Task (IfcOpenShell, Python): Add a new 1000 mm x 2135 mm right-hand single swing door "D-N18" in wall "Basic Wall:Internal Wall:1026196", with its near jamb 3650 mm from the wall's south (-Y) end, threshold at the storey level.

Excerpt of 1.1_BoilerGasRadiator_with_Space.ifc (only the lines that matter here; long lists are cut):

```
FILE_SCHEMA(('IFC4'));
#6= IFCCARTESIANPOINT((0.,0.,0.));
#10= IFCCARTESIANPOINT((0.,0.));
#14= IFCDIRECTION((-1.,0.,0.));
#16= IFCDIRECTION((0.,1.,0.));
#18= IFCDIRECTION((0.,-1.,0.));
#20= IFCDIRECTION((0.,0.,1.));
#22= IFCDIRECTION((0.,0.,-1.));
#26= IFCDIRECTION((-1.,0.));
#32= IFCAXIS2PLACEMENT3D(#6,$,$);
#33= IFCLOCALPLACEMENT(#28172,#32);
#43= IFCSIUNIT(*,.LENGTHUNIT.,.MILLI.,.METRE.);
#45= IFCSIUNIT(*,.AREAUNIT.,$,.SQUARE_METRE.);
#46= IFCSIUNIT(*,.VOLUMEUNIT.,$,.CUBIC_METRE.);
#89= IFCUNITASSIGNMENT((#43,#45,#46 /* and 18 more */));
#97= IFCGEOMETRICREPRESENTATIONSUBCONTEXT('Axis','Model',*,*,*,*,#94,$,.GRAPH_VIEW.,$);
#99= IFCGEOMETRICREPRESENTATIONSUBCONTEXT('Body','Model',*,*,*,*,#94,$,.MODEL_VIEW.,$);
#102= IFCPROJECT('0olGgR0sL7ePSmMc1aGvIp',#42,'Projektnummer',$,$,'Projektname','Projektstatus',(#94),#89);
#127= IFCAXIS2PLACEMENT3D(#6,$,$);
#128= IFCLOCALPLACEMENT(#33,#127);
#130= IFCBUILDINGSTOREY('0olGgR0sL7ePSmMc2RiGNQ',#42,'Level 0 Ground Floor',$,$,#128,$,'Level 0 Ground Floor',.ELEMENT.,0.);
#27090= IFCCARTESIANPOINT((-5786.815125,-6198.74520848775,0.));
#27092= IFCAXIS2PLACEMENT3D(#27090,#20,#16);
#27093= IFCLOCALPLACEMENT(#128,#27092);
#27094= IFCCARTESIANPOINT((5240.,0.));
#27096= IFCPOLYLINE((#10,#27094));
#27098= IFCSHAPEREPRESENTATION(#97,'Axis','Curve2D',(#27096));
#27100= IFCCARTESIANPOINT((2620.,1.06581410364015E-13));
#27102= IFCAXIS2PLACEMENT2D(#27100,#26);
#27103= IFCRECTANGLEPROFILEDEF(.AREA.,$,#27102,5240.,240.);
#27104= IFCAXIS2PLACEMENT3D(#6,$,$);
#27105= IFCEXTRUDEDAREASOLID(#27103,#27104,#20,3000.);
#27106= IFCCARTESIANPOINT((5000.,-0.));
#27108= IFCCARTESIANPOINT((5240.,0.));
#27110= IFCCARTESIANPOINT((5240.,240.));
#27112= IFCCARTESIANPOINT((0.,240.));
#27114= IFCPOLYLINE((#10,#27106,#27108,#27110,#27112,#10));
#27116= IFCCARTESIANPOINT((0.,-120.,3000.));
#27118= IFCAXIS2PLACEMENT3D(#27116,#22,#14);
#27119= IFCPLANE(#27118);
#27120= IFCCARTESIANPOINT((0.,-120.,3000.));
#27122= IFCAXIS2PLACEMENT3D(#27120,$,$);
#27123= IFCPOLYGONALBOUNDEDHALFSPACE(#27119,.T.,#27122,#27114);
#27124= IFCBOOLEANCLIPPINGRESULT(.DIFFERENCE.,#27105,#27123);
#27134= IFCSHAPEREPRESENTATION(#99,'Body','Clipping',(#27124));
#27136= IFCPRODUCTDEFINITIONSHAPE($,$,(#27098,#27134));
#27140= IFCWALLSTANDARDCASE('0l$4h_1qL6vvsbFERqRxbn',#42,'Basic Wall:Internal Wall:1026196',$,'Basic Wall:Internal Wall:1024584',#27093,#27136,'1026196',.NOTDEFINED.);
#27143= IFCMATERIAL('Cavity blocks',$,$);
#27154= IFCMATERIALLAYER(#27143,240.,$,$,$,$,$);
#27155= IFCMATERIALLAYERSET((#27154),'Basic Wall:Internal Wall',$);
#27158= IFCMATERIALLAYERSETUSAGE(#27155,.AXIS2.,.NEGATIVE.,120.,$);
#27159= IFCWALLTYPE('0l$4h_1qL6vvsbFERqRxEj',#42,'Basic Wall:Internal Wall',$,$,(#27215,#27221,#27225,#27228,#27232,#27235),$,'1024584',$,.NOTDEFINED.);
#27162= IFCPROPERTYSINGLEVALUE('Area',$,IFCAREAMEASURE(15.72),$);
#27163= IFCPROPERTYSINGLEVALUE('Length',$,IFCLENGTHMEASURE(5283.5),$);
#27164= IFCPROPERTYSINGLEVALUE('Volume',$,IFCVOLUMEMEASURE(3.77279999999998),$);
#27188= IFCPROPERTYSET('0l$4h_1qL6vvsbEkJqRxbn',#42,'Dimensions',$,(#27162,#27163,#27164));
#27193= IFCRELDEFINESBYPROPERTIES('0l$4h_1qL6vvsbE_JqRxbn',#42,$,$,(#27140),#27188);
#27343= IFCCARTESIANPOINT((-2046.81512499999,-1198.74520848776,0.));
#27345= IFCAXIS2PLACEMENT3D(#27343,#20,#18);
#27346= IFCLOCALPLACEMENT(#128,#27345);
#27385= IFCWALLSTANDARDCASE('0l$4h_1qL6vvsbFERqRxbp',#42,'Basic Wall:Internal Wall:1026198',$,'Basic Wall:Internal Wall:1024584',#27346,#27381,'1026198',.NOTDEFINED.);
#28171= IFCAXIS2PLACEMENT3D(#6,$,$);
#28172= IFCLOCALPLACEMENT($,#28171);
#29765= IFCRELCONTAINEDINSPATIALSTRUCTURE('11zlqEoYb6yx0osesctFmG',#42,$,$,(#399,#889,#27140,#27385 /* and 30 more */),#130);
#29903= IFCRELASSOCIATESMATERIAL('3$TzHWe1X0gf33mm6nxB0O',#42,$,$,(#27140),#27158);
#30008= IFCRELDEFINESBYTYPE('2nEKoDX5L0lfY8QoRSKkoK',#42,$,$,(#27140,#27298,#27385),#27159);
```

```python
import numpy as np
import ifcopenshell
import ifcopenshell.api.feature
import ifcopenshell.api.geometry
import ifcopenshell.api.pset
import ifcopenshell.api.root
import ifcopenshell.api.spatial
import ifcopenshell.geom
import ifcopenshell.util.element
import ifcopenshell.util.placement
import ifcopenshell.util.representation
import ifcopenshell.util.shape
import ifcopenshell.util.unit

model = ifcopenshell.open("1.1_BoilerGasRadiator_with_Space.ifc")
unit_scale = ifcopenshell.util.unit.calculate_unit_scale(model)
area_scale = ifcopenshell.util.unit.calculate_unit_scale(model, "AREAUNIT")
volume_scale = ifcopenshell.util.unit.calculate_unit_scale(model, "VOLUMEUNIT")
settings = ifcopenshell.geom.settings()


def volume(element):
    """Net volume in cubic metres, openings subtracted."""
    shape = ifcopenshell.geom.create_shape(settings, element)
    return ifcopenshell.util.shape.get_volume(shape.geometry)


wall = model.by_guid("0l$4h_1qL6vvsbFERqRxbn")
storey = ifcopenshell.util.element.get_container(wall, ifc_class="IfcBuildingStorey")
context = ifcopenshell.util.representation.get_context(model, "Model", "Body", "MODEL_VIEW")
before = volume(wall)

width, height, from_end, sill = 1, 2.135, 3.65, 0.0  # metres

# The wall runs along its own X axis, and the end named is its -X end.
wall_shape = ifcopenshell.geom.create_shape(settings, wall)
x, y, z = ifcopenshell.util.shape.get_vertices(wall_shape.geometry).T
start = x.min() + from_end
face, thickness = float(y.min()), float(y.max() - y.min())
wall_matrix = ifcopenshell.util.placement.get_local_placement(wall.ObjectPlacement)
level = ifcopenshell.util.placement.get_local_placement(storey.ObjectPlacement)[2, 3]


def in_wall(x, y):
    """Placement at x, y metres in the wall's axes, at sill height."""
    matrix = wall_matrix.copy()
    matrix[:, 3] = wall_matrix @ np.array([x / unit_scale, y / unit_scale, 0.0, 1.0])
    matrix[2, 3] = level + sill / unit_scale
    return matrix


# Opening: a box that overshoots both wall faces by 50 mm.
opening = ifcopenshell.api.root.create_entity(model, ifc_class="IfcOpeningElement", predefined_type="OPENING")
box = ifcopenshell.api.geometry.add_wall_representation(
    model, context=context, length=width, height=height, thickness=thickness + 0.1
)
ifcopenshell.api.geometry.assign_representation(model, product=opening, representation=box)
ifcopenshell.api.geometry.edit_object_placement(model, product=opening, matrix=in_wall(start, face - 0.05), is_si=False)
ifcopenshell.api.feature.add_feature(model, feature=opening, element=wall)

door = ifcopenshell.api.root.create_entity(model, ifc_class="IfcDoor", name="D-N18", predefined_type="DOOR")
door.OverallWidth, door.OverallHeight = width / unit_scale, height / unit_scale
door.OperationType = "SINGLE_SWING_RIGHT"
body = ifcopenshell.api.geometry.add_door_representation(
    model,
    context=context,
    overall_width=door.OverallWidth,
    overall_height=door.OverallHeight,
    operation_type="SINGLE_SWING_RIGHT",
    lining_properties={"LiningDepth": thickness / unit_scale, "ThresholdDepth": thickness / unit_scale},
)
ifcopenshell.api.geometry.assign_representation(model, product=door, representation=body)
ifcopenshell.api.spatial.assign_container(model, products=[door], relating_structure=storey)
ifcopenshell.api.feature.add_filling(model, opening=opening, element=door)

# The lining spans the wall, so the door starts at the wall face.
ifcopenshell.api.geometry.edit_object_placement(model, product=door, matrix=in_wall(start, face), is_si=False)

after = volume(wall)

# Update the wall's stored quantities.
pset = model.by_id(ifcopenshell.util.element.get_pset(wall, "Dimensions", should_inherit=False)["id"])
ifcopenshell.api.pset.edit_pset(model, pset=pset, properties={
    "Area": model.create_entity("IfcAreaMeasure", after / thickness / area_scale),
    "Volume": model.create_entity("IfcVolumeMeasure", after / volume_scale),
})

print(f"wall volume {before:.3f} -> {after:.3f} m3")

model.write("1.1_BoilerGasRadiator_with_Space-out.ifc")
```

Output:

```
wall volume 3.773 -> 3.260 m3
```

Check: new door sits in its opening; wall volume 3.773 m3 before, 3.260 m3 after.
